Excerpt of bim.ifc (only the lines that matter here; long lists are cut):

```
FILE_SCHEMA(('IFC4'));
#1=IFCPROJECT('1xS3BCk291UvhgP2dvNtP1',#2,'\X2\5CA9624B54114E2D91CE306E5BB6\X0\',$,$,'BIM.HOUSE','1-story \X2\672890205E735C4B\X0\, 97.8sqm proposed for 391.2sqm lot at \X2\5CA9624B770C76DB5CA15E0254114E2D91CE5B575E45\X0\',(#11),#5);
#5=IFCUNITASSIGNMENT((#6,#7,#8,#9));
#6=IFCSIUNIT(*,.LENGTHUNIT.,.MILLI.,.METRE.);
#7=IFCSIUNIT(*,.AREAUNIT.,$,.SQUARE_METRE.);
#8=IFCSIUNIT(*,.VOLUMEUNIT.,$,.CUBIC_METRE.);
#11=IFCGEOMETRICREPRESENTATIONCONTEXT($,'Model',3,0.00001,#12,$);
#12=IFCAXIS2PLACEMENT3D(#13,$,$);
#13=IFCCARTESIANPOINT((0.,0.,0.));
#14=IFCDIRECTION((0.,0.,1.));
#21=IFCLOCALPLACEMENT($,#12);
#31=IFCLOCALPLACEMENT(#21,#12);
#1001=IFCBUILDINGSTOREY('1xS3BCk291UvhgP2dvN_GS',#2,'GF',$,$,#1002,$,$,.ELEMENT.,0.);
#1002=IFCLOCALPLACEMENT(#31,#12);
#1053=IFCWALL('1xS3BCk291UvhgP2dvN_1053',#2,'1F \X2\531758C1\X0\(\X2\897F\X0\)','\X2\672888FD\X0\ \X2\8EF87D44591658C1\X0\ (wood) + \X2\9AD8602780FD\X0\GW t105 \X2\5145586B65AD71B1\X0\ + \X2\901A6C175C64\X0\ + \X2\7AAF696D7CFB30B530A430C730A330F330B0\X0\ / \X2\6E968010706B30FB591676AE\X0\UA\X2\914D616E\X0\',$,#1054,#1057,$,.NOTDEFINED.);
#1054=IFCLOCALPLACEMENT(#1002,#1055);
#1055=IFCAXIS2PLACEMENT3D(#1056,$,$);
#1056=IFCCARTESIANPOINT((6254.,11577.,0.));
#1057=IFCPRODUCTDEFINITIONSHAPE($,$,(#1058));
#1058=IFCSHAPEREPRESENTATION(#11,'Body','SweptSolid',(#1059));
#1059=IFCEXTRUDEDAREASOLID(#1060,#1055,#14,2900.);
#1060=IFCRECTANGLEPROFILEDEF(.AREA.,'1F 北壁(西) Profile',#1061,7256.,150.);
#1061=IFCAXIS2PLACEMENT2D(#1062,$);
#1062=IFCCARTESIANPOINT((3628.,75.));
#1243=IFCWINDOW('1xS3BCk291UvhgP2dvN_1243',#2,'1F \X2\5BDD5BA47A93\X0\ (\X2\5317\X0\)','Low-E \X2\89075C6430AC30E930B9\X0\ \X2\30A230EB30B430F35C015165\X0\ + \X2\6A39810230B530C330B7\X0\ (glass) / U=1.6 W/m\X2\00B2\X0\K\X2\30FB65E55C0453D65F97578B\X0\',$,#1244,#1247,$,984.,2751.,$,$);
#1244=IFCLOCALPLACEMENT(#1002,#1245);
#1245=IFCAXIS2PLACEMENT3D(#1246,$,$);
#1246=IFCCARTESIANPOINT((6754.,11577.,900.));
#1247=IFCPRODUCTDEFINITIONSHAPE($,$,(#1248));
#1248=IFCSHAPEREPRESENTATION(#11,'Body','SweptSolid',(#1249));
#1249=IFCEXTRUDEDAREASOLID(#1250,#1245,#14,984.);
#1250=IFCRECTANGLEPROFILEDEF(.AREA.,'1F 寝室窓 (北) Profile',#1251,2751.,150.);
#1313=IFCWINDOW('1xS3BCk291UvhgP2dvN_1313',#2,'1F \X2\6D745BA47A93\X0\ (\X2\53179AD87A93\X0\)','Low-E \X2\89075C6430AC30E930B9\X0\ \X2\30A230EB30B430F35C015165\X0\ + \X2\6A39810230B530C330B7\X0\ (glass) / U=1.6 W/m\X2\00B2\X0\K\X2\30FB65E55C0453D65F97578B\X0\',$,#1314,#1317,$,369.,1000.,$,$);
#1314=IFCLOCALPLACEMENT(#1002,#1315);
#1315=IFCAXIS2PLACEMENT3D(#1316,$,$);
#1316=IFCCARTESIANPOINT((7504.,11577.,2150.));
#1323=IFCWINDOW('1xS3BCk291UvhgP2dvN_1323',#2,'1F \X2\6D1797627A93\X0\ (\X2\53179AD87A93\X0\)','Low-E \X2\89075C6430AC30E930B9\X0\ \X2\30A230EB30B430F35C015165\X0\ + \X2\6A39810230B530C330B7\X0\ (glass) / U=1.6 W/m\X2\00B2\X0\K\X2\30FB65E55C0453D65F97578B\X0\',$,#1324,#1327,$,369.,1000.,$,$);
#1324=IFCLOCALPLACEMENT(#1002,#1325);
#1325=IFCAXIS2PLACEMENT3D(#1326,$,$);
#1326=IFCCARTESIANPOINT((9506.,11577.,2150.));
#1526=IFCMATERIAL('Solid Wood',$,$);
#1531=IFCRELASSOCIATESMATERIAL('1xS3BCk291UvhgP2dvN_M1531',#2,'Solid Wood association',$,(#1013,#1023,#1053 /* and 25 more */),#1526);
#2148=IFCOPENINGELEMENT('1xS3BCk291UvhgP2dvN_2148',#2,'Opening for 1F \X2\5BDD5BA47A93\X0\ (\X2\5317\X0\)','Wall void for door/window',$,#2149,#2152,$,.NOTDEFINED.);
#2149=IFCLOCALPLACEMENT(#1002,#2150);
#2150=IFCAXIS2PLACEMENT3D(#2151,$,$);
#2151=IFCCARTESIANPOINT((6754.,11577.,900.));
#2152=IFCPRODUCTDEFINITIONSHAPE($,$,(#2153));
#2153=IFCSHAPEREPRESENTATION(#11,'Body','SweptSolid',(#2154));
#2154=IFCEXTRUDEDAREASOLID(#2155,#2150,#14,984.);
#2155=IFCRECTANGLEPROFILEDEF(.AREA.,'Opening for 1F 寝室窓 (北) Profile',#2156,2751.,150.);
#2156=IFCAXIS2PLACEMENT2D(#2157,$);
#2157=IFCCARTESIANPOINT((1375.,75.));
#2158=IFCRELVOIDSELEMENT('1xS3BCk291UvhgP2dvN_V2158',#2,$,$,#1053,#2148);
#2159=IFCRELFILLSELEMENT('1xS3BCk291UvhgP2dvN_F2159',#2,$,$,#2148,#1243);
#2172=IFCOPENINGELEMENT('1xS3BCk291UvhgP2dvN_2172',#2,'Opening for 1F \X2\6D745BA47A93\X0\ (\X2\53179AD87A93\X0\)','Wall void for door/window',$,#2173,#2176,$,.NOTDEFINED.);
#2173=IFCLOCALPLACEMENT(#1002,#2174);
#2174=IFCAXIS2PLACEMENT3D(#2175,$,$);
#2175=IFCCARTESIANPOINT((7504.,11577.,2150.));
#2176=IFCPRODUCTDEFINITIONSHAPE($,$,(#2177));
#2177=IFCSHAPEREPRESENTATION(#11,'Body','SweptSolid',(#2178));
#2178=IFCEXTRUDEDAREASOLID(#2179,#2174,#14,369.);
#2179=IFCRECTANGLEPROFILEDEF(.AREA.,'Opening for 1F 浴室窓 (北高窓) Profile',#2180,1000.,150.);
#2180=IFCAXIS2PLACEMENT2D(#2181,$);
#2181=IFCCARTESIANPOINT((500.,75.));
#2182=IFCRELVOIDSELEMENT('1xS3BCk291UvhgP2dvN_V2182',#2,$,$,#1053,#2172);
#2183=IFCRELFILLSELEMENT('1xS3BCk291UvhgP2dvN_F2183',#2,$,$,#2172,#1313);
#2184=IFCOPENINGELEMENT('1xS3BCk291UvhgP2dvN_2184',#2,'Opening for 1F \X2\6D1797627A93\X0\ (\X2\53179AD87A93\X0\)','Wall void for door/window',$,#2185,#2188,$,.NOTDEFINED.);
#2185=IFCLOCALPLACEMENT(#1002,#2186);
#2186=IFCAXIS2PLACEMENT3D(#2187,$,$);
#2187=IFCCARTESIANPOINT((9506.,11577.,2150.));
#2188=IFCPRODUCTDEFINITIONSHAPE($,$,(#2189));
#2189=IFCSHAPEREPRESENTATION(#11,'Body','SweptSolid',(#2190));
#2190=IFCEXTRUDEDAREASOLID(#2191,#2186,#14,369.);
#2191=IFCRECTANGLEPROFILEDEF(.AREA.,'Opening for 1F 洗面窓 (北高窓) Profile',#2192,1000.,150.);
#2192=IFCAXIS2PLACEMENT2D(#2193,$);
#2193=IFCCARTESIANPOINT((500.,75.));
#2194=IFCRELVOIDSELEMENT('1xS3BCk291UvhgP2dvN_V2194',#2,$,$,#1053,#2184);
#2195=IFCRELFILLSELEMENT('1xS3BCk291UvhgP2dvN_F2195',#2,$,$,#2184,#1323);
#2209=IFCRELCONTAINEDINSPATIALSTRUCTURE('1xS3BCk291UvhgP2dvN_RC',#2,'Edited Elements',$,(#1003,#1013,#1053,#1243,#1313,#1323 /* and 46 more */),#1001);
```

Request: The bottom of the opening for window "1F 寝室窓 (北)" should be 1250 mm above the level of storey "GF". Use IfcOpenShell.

```python
import numpy as np
import ifcopenshell
import ifcopenshell.api.geometry
import ifcopenshell.geom
import ifcopenshell.util.element
import ifcopenshell.util.placement
import ifcopenshell.util.shape
import ifcopenshell.util.unit

model = ifcopenshell.open("bim.ifc")
unit_scale = ifcopenshell.util.unit.calculate_unit_scale(model)

window = model.by_guid("1xS3BCk291UvhgP2dvN_1243")
opening = window.FillsVoids[0].RelatingOpeningElement
storey = ifcopenshell.util.element.get_container(window, ifc_class="IfcBuildingStorey")
level = ifcopenshell.util.placement.get_local_placement(storey.ObjectPlacement)[2, 3]

# The opening's origin need not be at the sill, so measure its lowest point.
shape = ifcopenshell.geom.create_shape(ifcopenshell.geom.settings(), opening)
bottom = ifcopenshell.util.shape.get_shape_bottom_elevation(shape, shape.geometry) / unit_scale
dz = level + 1250.0 - bottom

shift = np.array([0.0, 0.0, dz])
# The window is not placed relative to its opening, so move both.
for product in (opening, window):
    matrix = ifcopenshell.util.placement.get_local_placement(product.ObjectPlacement)
    matrix[:3, 3] += shift
    ifcopenshell.api.geometry.edit_object_placement(model, product=product, matrix=matrix, is_si=False)

print(f"moved by {dz * unit_scale:+.3f} m")

model.write("bim_edited.ifc")
```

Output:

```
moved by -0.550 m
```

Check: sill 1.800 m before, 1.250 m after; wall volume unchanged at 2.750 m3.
